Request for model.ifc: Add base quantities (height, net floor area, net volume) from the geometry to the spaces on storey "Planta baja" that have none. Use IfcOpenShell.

First a look at what the model holds.

```python
import ifcopenshell
import ifcopenshell.util.element
import ifcopenshell.util.unit

model = ifcopenshell.open("model.ifc")
print(model.schema)
for unit_type in ("LENGTHUNIT", "AREAUNIT", "VOLUMEUNIT"):
    print(unit_type, ifcopenshell.util.unit.calculate_unit_scale(model, unit_type))
storey = next(s for s in model.by_type("IfcBuildingStorey") if s.Name == "Planta baja")
spaces = [e for e in ifcopenshell.util.element.get_decomposition(storey) if e.is_a("IfcSpace")]
for e in sorted(spaces, key=lambda e: e.id()):
    print(e.id(), e.is_a(), e.Name, list(ifcopenshell.util.element.get_psets(e, qtos_only=True)), sep=" | ")
```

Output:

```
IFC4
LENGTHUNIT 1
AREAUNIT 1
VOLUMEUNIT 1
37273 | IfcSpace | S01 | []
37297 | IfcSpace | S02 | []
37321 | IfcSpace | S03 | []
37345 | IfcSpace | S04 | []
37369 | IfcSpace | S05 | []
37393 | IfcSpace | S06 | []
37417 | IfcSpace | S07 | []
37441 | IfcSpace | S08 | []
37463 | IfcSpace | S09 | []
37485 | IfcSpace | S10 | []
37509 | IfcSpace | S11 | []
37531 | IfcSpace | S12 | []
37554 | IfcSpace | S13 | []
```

```python
import ifcopenshell
import ifcopenshell.api.pset
import ifcopenshell.geom
import ifcopenshell.util.element
import ifcopenshell.util.shape
import ifcopenshell.util.unit

model = ifcopenshell.open("model.ifc")
unit_scale = ifcopenshell.util.unit.calculate_unit_scale(model)
area_scale = ifcopenshell.util.unit.calculate_unit_scale(model, "AREAUNIT")
volume_scale = ifcopenshell.util.unit.calculate_unit_scale(model, "VOLUMEUNIT")
settings = ifcopenshell.geom.settings()

storey = next(s for s in model.by_type("IfcBuildingStorey") if s.Name == "Planta baja")
spaces = [e for e in ifcopenshell.util.element.get_decomposition(storey) if e.is_a("IfcSpace")]

for e in sorted(spaces, key=lambda e: e.id()):
    if ifcopenshell.util.element.get_psets(e, qtos_only=True, should_inherit=False):
        continue
    # Geometry comes back in metres, in the element's own axes.
    shape = ifcopenshell.geom.create_shape(settings, e)
    values = {
        "Height": ifcopenshell.util.shape.get_z(shape.geometry) / unit_scale,
        "NetFloorArea": ifcopenshell.util.shape.get_footprint_area(shape.geometry) / area_scale,
        "NetVolume": ifcopenshell.util.shape.get_volume(shape.geometry) / volume_scale,
    }
    qto = ifcopenshell.api.pset.add_qto(model, product=e, name="Qto_SpaceBaseQuantities")
    ifcopenshell.api.pset.edit_qto(model, qto=qto, properties=values)
    print(e.id(), {k: round(v, 3) for k, v in values.items()})

model.write("model_v2.ifc")
```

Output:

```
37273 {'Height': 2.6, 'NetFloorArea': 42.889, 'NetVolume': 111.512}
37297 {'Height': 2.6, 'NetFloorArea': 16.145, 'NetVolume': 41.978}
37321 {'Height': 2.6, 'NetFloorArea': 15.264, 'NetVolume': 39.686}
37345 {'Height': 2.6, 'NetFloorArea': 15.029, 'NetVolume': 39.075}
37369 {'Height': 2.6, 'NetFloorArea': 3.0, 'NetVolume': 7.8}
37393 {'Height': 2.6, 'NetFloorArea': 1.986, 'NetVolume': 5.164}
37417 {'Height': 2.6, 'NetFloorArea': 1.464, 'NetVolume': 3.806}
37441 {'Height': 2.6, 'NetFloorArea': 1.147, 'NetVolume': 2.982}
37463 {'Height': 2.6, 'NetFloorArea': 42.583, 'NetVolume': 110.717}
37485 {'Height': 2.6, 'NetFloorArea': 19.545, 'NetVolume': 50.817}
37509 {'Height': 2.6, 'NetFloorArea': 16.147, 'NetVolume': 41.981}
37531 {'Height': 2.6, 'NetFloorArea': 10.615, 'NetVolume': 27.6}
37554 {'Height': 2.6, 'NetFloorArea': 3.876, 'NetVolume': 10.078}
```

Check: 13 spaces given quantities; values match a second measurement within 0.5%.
